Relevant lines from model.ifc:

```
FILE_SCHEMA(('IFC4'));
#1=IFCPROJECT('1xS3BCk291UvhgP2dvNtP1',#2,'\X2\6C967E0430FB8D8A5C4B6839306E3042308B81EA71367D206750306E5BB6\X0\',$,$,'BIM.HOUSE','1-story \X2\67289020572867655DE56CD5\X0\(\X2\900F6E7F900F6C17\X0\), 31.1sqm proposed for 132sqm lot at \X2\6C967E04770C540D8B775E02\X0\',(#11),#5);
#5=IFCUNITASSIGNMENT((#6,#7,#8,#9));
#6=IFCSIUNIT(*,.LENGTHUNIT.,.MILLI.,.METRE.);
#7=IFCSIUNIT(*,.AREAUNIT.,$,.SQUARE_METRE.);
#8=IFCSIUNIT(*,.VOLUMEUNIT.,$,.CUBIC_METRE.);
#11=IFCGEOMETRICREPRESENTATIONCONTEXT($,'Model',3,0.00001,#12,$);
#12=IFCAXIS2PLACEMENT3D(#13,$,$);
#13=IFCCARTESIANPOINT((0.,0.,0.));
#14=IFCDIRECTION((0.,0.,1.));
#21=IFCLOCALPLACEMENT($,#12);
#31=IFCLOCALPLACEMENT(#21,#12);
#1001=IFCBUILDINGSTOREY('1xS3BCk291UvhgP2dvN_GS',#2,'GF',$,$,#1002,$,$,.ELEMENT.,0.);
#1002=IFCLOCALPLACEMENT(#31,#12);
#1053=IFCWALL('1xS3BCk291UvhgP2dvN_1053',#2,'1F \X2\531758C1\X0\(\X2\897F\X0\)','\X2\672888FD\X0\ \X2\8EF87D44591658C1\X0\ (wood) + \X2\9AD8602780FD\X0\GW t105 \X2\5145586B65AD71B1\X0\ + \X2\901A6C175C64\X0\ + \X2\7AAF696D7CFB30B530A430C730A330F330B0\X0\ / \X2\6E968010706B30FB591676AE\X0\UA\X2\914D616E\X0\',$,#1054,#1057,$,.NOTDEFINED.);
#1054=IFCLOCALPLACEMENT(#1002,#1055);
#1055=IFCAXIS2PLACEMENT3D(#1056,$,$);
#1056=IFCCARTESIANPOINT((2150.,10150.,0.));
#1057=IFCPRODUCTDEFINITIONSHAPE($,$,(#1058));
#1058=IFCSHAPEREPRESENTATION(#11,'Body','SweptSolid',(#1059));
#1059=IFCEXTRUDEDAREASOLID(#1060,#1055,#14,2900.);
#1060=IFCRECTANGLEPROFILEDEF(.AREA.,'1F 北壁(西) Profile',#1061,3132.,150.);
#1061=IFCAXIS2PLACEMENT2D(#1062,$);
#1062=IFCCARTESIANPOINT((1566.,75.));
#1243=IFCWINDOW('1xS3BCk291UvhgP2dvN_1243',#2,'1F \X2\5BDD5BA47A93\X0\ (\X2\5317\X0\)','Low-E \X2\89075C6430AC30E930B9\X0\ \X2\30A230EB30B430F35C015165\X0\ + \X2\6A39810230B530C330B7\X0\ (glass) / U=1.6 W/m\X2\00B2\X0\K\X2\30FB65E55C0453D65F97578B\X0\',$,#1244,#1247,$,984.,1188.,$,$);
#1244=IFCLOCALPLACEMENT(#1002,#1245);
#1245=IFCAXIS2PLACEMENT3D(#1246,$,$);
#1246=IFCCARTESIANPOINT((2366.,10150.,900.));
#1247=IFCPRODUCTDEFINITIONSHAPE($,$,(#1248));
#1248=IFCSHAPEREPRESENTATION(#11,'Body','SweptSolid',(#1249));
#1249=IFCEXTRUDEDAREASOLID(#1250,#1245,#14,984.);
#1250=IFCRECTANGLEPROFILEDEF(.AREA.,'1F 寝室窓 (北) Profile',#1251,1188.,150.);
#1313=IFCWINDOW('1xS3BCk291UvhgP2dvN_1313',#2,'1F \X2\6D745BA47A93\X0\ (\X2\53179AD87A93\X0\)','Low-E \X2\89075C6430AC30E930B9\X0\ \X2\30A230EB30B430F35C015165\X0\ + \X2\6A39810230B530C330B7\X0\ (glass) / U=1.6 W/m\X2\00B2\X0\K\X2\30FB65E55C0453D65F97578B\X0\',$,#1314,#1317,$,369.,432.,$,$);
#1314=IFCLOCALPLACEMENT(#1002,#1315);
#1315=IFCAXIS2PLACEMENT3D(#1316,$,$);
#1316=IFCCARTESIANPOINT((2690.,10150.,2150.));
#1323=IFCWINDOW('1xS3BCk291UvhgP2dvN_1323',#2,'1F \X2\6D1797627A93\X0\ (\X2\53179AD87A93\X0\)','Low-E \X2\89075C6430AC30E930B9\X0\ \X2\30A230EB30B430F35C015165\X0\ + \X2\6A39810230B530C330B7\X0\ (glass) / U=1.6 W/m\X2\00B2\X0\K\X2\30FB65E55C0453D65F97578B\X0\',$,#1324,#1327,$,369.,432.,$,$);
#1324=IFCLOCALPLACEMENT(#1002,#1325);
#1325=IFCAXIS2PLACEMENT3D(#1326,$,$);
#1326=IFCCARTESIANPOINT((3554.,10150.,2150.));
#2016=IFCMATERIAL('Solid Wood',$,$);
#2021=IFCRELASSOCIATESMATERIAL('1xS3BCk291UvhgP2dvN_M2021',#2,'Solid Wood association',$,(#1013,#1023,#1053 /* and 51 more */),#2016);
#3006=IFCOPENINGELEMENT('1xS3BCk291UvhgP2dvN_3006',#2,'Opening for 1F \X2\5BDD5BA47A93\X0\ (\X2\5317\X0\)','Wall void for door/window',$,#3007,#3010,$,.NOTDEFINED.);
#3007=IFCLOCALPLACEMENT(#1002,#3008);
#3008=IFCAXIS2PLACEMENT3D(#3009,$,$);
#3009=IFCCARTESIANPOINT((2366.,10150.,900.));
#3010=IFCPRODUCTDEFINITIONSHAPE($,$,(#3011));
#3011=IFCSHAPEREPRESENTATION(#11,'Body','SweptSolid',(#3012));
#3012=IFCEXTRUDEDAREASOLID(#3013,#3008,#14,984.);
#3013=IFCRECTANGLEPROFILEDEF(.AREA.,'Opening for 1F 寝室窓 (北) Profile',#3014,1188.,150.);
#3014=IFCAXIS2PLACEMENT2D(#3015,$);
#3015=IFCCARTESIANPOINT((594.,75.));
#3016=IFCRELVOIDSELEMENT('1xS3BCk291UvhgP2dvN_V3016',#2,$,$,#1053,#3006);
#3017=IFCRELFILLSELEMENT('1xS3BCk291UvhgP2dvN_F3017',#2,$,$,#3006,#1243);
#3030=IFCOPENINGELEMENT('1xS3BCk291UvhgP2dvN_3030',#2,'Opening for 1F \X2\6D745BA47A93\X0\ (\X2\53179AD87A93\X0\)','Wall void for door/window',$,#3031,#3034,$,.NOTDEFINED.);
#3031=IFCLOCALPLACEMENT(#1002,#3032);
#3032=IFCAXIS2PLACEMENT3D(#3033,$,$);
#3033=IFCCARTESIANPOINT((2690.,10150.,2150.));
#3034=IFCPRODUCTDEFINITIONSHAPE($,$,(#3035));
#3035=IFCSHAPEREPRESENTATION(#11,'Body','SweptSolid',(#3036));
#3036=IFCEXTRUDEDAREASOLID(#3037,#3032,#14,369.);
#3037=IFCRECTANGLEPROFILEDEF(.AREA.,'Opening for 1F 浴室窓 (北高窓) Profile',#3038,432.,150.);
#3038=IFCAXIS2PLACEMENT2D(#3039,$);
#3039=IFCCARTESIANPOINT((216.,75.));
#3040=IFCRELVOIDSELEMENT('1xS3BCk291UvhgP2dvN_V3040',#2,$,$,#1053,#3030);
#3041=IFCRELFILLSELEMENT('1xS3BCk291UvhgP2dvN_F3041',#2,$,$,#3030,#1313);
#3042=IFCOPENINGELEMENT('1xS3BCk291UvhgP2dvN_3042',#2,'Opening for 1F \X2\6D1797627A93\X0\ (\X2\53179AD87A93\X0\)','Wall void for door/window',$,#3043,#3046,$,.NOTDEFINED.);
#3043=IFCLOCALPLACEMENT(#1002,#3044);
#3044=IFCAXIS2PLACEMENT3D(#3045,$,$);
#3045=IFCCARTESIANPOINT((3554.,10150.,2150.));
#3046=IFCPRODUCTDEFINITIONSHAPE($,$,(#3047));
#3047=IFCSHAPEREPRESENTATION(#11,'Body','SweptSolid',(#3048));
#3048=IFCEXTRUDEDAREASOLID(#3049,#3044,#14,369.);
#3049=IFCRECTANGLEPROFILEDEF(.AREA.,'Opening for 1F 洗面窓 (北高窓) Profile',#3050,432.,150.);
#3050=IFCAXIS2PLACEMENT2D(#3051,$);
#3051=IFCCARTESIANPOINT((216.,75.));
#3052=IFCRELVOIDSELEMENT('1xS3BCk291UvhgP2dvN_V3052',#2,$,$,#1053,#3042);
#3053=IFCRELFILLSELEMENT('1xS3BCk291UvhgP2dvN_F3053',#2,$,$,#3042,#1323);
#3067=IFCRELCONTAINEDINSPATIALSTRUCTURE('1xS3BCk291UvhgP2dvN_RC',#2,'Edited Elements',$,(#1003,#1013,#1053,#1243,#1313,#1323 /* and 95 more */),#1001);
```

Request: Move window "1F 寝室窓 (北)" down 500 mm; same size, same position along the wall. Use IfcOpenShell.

```python
import numpy as np
import ifcopenshell
import ifcopenshell.api.geometry
import ifcopenshell.util.placement
import ifcopenshell.util.unit

model = ifcopenshell.open("model.ifc")
unit_scale = ifcopenshell.util.unit.calculate_unit_scale(model)

window = model.by_id(1243)
opening = window.FillsVoids[0].RelatingOpeningElement
dz = -0.5 / unit_scale

shift = np.array([0.0, 0.0, dz])
# The window is not placed relative to its opening, so move both.
for product in (opening, window):
    matrix = ifcopenshell.util.placement.get_local_placement(product.ObjectPlacement)
    matrix[:3, 3] += shift
    ifcopenshell.api.geometry.edit_object_placement(model, product=product, matrix=matrix, is_si=False)

print(f"moved by {dz * unit_scale:+.3f} m")

model.write("model_v2.ifc")
```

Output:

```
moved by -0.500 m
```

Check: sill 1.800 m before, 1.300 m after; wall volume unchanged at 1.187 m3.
